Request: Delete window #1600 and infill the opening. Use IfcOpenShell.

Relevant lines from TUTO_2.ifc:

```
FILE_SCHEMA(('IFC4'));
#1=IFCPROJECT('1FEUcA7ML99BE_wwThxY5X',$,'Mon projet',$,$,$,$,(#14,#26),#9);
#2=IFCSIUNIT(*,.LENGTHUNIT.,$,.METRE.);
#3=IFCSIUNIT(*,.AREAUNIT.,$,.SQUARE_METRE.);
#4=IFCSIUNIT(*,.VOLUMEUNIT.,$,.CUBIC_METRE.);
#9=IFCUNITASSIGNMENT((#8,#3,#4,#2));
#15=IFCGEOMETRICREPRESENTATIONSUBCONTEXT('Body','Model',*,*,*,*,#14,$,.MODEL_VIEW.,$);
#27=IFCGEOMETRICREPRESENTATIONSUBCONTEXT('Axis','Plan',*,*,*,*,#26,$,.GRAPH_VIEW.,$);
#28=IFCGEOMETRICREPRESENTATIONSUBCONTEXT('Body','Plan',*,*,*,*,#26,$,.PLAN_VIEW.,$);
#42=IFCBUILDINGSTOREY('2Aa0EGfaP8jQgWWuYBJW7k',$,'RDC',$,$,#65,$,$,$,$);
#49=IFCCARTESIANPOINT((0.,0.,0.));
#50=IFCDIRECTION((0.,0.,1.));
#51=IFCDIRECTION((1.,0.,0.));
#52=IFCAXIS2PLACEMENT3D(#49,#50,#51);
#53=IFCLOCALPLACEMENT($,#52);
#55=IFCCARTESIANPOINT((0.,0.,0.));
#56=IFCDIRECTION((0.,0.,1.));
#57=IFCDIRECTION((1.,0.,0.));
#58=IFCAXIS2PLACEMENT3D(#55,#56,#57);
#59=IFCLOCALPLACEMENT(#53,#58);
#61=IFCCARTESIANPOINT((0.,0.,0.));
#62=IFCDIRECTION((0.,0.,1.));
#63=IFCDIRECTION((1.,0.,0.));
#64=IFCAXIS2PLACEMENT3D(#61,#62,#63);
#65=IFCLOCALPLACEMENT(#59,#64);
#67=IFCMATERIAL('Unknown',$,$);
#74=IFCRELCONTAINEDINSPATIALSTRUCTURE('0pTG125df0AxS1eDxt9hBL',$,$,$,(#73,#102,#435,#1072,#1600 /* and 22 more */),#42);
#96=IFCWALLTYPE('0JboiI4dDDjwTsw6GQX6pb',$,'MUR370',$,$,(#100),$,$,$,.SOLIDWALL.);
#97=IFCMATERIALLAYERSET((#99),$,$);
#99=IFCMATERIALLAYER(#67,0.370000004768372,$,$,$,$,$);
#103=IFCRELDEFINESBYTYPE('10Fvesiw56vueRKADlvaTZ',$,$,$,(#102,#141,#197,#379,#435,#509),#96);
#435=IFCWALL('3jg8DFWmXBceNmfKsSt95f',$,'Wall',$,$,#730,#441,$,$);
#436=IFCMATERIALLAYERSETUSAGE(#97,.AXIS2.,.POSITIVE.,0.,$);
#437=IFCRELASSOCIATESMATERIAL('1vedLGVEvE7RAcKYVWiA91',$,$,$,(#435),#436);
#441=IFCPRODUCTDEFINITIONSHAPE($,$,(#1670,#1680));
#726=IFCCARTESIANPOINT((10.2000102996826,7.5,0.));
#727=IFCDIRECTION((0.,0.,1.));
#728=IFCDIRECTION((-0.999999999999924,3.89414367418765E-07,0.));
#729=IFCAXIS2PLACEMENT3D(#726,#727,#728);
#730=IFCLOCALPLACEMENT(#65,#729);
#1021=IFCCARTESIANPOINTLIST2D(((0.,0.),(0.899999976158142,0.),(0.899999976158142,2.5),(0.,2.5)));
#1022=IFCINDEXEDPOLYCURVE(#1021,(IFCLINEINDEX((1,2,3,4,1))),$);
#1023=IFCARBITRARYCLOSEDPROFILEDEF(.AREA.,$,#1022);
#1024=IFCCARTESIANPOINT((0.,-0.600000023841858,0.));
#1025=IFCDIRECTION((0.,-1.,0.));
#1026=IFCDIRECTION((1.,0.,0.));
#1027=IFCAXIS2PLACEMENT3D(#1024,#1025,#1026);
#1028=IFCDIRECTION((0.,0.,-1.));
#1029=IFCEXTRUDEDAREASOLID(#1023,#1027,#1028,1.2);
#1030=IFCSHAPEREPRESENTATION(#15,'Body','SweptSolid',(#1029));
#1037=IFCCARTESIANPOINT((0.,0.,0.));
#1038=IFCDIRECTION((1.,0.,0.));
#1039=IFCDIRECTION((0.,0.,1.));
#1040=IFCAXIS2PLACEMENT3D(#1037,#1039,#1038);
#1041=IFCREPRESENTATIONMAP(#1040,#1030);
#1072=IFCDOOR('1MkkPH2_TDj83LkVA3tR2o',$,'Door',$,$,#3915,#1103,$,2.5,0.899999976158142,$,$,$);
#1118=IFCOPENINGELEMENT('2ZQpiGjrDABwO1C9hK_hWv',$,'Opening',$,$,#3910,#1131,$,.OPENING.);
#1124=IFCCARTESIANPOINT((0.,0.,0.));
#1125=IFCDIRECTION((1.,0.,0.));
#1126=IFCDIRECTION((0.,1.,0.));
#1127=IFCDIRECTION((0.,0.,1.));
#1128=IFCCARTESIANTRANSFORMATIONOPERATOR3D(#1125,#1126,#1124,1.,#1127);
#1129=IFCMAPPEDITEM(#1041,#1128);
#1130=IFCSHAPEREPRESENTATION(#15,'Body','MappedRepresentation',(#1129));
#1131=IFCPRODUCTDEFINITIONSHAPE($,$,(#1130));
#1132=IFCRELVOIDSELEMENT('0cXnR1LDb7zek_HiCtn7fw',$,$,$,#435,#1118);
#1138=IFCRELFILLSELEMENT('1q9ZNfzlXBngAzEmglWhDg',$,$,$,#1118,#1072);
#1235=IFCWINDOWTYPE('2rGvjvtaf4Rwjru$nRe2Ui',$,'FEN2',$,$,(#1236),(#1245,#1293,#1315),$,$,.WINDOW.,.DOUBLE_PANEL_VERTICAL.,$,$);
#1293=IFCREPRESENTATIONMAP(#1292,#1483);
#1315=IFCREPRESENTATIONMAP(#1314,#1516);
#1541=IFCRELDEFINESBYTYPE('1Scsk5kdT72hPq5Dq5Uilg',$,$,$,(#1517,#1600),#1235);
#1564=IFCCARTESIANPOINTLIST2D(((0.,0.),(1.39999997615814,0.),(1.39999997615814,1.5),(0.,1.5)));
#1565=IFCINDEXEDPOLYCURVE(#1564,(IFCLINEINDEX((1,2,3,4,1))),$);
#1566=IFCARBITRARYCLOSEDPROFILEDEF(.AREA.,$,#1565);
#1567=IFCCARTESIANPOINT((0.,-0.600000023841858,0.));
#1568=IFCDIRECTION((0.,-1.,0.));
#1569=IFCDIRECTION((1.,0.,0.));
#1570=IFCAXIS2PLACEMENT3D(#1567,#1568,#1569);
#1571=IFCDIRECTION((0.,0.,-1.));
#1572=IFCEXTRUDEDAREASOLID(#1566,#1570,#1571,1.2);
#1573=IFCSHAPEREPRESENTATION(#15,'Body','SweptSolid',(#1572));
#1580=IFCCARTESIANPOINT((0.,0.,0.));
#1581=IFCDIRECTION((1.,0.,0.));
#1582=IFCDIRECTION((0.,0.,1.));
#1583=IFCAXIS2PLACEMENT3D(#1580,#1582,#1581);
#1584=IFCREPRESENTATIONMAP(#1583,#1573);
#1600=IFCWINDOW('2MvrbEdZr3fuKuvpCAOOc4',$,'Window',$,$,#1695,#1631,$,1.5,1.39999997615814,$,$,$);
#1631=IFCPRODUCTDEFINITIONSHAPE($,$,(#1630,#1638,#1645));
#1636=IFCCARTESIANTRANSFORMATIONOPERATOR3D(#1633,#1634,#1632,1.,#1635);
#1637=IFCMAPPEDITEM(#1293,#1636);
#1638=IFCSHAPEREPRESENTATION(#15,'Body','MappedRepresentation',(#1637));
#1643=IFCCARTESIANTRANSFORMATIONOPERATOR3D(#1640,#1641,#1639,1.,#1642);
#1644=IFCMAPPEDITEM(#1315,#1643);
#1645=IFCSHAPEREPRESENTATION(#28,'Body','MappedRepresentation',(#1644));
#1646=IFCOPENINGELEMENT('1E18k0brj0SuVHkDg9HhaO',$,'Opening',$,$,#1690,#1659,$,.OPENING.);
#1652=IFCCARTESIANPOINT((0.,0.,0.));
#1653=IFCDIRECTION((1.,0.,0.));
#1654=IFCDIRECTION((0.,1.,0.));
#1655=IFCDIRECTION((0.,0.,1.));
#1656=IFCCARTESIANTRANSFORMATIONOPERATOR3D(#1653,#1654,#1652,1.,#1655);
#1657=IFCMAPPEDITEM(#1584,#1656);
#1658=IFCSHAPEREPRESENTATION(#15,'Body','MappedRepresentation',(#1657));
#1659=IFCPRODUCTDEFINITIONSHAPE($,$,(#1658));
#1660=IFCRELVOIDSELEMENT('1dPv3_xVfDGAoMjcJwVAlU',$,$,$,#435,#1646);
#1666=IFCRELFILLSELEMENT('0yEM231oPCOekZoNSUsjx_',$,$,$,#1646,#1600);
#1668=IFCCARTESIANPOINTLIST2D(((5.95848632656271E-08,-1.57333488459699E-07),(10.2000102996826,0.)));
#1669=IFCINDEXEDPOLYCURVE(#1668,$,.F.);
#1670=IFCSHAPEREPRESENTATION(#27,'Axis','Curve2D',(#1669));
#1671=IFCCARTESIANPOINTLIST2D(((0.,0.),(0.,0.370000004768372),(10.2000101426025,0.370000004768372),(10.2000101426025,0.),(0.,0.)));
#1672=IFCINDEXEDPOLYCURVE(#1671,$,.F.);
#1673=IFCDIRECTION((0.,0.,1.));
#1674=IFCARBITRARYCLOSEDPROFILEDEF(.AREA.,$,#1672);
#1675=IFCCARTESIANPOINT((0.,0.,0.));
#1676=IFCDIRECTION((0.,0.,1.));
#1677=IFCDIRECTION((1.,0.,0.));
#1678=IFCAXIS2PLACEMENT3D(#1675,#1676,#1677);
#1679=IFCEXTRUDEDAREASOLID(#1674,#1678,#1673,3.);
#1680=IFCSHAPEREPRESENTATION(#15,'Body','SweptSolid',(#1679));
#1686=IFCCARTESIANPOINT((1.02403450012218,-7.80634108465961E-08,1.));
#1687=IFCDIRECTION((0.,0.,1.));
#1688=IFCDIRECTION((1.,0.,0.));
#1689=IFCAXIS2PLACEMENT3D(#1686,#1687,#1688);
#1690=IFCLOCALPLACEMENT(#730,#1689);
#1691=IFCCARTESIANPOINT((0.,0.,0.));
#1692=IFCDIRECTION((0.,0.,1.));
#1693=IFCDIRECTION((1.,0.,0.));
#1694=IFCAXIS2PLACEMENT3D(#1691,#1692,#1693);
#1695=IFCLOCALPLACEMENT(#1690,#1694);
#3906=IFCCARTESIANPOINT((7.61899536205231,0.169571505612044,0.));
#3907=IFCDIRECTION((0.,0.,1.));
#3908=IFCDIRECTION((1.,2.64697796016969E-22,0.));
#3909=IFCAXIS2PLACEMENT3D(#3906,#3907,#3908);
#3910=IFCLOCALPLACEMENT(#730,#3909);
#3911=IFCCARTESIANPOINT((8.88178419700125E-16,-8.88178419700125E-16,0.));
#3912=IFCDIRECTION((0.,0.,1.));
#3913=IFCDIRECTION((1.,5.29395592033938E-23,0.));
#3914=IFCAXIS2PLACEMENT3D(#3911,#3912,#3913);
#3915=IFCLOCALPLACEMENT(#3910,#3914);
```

```python
import ifcopenshell
import ifcopenshell.api.feature
import ifcopenshell.api.root
import ifcopenshell.geom
import ifcopenshell.util.shape

model = ifcopenshell.open("TUTO_2.ifc")
settings = ifcopenshell.geom.settings()


def volume(element):
    """Net volume in cubic metres, openings subtracted."""
    shape = ifcopenshell.geom.create_shape(settings, element)
    return ifcopenshell.util.shape.get_volume(shape.geometry)


window = model.by_guid("2MvrbEdZr3fuKuvpCAOOc4")
opening = window.FillsVoids[0].RelatingOpeningElement
wall = opening.VoidsElements[0].RelatingBuildingElement
before = volume(wall)

ifcopenshell.api.root.remove_product(model, product=window)
ifcopenshell.api.feature.remove_feature(model, feature=opening)

after = volume(wall)

print(f"wall volume {before:.3f} -> {after:.3f} m3")

model.write("TUTO_2_rev.ifc")
```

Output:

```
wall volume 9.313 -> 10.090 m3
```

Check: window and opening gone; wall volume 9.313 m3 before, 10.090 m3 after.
